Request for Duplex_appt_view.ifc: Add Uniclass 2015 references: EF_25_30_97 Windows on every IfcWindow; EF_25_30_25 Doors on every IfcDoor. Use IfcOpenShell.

First a look at what the model holds.

```python
import ifcopenshell

model = ifcopenshell.open("Duplex_appt_view.ifc")
print(model.schema)
print("classifications:", [c.Name for c in model.by_type("IfcClassification")])
for ifc_class in ("IfcDoor", "IfcRoof", "IfcStair", "IfcWall", "IfcWindow"):
    print(ifc_class, len(model.by_type(ifc_class)))
```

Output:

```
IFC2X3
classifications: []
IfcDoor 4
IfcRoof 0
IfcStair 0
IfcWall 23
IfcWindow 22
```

```python
import ifcopenshell
import ifcopenshell.api.classification

model = ifcopenshell.open("Duplex_appt_view.ifc")

# IFC2X3 requires Source and Edition and has no link from the project to the system.
system = model.create_entity("IfcClassification", Source="NBS", Edition="2015", Name="Uniclass 2015")

codes = {
    "IfcWindow": ("EF_25_30_97", "Windows"),
    "IfcDoor": ("EF_25_30_25", "Doors"),
}
for ifc_class, (code, name) in codes.items():
    products = model.by_type(ifc_class)
    ifcopenshell.api.classification.add_reference(
        model, products=products, classification=system, identification=code, name=name
    )
    print(code, len(products))

model.write("Duplex_appt_view_v2.ifc")
```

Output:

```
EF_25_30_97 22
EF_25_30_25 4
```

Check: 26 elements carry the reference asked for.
